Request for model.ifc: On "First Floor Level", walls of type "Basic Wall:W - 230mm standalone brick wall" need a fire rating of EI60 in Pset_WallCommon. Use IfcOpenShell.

First a look at what the model holds.

```python
import ifcopenshell
import ifcopenshell.util.element

model = ifcopenshell.open("model.ifc")
print(model.schema)
storey = next(s for s in model.by_type("IfcBuildingStorey") if s.Name == "First Floor Level")
walls = [e for e in ifcopenshell.util.element.get_decomposition(storey) if e.is_a("IfcWall")]
seen = {}
for e in walls:
    element_type = ifcopenshell.util.element.get_type(e)
    key = (element_type.Name if element_type != e and element_type else None, ifcopenshell.util.element.get_pset(e, "Pset_WallCommon", "FireRating"))
    seen[key] = seen.get(key, 0) + 1
for (name, value), count in sorted(seen.items(), key=str):
    print(count, "x", name, "|", value)
```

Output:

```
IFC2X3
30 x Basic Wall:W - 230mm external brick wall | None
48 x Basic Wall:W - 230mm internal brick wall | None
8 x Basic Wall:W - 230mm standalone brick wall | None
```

```python
import ifcopenshell
import ifcopenshell.api.pset
import ifcopenshell.util.element

model = ifcopenshell.open("model.ifc")

storey = next(s for s in model.by_type("IfcBuildingStorey") if s.Name == "First Floor Level")
walls = [e for e in ifcopenshell.util.element.get_decomposition(storey) if e.is_a("IfcWall")]

count = 0
for e in walls:
    element_type = ifcopenshell.util.element.get_type(e)
    if element_type in (None, e) or element_type.Name != "Basic Wall:W - 230mm standalone brick wall":
        continue
    # add_pset returns the element's existing set when there is one.
    pset = ifcopenshell.api.pset.add_pset(model, product=e, name="Pset_WallCommon")
    ifcopenshell.api.pset.edit_pset(model, pset=pset, properties={"FireRating": "EI60"})
    count += 1

print(count, "walls updated")

model.write("model_rev.ifc")
```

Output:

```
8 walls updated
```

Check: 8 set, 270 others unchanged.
